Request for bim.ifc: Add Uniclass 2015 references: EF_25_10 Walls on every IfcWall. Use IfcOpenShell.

First a look at what the model holds.

```python
import ifcopenshell

model = ifcopenshell.open("bim.ifc")
print(model.schema)
print("classifications:", [c.Name for c in model.by_type("IfcClassification")])
for ifc_class in ("IfcDoor", "IfcRoof", "IfcStair", "IfcWall", "IfcWindow"):
    print(ifc_class, len(model.by_type(ifc_class)))
```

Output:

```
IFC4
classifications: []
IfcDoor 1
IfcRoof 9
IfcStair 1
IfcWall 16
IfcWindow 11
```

```python
import ifcopenshell
import ifcopenshell.api.classification

model = ifcopenshell.open("bim.ifc")

system = ifcopenshell.api.classification.add_classification(model, classification="Uniclass 2015")

codes = {
    "IfcWall": ("EF_25_10", "Walls"),
}
for ifc_class, (code, name) in codes.items():
    products = model.by_type(ifc_class)
    ifcopenshell.api.classification.add_reference(
        model, products=products, classification=system, identification=code, name=name
    )
    print(code, len(products))

model.write("bim_v2.ifc")
```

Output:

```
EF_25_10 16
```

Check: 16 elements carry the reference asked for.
